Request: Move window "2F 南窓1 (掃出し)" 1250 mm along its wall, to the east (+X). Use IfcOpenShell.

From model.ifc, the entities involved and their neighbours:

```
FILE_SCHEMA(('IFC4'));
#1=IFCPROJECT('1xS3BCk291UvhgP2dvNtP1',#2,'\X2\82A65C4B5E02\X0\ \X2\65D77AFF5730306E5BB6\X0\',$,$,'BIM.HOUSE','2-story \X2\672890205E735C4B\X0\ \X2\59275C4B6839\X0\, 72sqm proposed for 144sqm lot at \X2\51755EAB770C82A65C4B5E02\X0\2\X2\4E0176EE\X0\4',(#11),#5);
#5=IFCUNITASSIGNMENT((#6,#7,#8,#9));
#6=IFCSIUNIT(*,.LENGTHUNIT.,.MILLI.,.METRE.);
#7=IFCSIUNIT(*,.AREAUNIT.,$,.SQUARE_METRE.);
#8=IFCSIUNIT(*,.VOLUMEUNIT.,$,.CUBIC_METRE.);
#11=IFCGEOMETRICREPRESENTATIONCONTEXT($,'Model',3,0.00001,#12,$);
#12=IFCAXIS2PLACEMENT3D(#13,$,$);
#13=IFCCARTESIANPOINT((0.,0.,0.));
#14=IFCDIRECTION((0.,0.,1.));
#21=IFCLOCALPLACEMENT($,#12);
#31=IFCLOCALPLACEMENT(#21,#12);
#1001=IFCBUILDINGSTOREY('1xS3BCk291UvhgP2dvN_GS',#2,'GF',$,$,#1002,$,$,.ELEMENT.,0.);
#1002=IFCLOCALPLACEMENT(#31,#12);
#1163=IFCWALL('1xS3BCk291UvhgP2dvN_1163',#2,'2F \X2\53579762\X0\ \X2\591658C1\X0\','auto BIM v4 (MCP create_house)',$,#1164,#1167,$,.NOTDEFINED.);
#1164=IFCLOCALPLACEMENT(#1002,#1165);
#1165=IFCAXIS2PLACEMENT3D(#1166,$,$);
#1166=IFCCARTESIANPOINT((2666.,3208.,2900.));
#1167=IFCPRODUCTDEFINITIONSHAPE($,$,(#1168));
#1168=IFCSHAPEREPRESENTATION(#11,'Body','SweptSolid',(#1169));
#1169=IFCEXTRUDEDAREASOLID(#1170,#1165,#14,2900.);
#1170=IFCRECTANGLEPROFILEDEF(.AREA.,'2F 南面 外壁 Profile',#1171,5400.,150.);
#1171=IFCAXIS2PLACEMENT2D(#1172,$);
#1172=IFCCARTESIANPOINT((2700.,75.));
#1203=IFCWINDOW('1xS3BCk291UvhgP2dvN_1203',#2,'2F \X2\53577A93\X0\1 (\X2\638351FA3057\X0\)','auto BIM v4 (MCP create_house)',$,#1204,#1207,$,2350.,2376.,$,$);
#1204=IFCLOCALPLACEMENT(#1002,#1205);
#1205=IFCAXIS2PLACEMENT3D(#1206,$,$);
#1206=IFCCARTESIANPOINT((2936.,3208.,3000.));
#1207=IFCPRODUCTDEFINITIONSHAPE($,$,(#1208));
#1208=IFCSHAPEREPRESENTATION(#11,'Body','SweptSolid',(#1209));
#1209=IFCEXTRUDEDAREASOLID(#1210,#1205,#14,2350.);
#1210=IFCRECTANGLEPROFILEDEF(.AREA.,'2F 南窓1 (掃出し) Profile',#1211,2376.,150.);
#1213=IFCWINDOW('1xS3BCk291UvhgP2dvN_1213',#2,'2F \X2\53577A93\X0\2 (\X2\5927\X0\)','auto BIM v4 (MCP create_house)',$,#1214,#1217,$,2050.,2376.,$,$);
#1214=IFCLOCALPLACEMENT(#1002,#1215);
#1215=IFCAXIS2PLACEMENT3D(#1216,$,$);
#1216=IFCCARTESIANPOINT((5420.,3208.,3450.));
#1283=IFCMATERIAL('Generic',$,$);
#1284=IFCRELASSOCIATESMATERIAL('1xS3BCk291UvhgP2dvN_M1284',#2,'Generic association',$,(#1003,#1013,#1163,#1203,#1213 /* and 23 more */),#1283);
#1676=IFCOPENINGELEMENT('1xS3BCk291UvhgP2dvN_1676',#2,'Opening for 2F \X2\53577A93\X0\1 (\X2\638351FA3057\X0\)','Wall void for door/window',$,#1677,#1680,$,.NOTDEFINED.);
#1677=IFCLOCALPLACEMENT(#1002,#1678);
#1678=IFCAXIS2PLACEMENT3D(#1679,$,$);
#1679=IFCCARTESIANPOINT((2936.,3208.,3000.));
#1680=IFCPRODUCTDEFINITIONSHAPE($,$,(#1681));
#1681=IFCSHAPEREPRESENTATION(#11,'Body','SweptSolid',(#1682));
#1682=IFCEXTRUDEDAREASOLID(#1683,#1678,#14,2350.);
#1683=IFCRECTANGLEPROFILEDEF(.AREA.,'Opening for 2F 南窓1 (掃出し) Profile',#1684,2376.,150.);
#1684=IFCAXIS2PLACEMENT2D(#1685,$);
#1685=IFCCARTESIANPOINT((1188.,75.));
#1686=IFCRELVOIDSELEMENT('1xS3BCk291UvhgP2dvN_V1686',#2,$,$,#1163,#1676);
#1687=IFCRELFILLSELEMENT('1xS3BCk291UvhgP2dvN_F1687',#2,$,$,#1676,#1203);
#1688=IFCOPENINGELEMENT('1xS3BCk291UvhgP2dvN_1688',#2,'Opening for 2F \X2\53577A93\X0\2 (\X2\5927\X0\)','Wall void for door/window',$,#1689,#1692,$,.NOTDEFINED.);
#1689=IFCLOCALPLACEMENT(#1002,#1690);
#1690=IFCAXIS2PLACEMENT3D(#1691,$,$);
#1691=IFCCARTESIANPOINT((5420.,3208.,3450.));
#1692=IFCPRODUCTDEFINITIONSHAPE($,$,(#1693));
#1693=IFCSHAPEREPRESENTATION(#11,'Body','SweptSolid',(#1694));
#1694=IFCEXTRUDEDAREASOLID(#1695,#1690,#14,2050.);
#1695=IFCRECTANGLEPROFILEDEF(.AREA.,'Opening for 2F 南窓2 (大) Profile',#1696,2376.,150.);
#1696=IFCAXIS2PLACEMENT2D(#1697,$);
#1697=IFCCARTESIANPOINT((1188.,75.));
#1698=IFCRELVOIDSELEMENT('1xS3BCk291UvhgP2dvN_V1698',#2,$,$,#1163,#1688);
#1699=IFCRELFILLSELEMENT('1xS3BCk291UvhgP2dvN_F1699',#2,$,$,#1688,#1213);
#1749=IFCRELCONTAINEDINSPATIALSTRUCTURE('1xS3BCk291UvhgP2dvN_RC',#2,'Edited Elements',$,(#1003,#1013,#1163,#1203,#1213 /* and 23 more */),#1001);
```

```python
import ifcopenshell
import ifcopenshell.api.geometry
import ifcopenshell.util.placement
import ifcopenshell.util.unit

model = ifcopenshell.open("model.ifc")
unit_scale = ifcopenshell.util.unit.calculate_unit_scale(model)

window = model.by_guid("1xS3BCk291UvhgP2dvN_1203")
opening = window.FillsVoids[0].RelatingOpeningElement
wall = opening.VoidsElements[0].RelatingBuildingElement

wall_matrix = ifcopenshell.util.placement.get_local_placement(wall.ObjectPlacement)
shift = wall_matrix[:3, 0] * 1.25 / unit_scale
before = ifcopenshell.util.placement.get_local_placement(window.ObjectPlacement)[:3, 3].copy()

# The window is not placed relative to its opening, so move both.
for product in (opening, window):
    matrix = ifcopenshell.util.placement.get_local_placement(product.ObjectPlacement)
    matrix[:3, 3] += shift
    ifcopenshell.api.geometry.edit_object_placement(model, product=product, matrix=matrix, is_si=False)

after = ifcopenshell.util.placement.get_local_placement(window.ObjectPlacement)[:3, 3]
print("window moved by", (after - before).round(3) + 0.0)

model.write("model_v2.ifc")
```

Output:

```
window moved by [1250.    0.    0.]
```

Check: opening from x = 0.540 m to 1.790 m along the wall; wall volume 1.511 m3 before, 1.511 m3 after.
